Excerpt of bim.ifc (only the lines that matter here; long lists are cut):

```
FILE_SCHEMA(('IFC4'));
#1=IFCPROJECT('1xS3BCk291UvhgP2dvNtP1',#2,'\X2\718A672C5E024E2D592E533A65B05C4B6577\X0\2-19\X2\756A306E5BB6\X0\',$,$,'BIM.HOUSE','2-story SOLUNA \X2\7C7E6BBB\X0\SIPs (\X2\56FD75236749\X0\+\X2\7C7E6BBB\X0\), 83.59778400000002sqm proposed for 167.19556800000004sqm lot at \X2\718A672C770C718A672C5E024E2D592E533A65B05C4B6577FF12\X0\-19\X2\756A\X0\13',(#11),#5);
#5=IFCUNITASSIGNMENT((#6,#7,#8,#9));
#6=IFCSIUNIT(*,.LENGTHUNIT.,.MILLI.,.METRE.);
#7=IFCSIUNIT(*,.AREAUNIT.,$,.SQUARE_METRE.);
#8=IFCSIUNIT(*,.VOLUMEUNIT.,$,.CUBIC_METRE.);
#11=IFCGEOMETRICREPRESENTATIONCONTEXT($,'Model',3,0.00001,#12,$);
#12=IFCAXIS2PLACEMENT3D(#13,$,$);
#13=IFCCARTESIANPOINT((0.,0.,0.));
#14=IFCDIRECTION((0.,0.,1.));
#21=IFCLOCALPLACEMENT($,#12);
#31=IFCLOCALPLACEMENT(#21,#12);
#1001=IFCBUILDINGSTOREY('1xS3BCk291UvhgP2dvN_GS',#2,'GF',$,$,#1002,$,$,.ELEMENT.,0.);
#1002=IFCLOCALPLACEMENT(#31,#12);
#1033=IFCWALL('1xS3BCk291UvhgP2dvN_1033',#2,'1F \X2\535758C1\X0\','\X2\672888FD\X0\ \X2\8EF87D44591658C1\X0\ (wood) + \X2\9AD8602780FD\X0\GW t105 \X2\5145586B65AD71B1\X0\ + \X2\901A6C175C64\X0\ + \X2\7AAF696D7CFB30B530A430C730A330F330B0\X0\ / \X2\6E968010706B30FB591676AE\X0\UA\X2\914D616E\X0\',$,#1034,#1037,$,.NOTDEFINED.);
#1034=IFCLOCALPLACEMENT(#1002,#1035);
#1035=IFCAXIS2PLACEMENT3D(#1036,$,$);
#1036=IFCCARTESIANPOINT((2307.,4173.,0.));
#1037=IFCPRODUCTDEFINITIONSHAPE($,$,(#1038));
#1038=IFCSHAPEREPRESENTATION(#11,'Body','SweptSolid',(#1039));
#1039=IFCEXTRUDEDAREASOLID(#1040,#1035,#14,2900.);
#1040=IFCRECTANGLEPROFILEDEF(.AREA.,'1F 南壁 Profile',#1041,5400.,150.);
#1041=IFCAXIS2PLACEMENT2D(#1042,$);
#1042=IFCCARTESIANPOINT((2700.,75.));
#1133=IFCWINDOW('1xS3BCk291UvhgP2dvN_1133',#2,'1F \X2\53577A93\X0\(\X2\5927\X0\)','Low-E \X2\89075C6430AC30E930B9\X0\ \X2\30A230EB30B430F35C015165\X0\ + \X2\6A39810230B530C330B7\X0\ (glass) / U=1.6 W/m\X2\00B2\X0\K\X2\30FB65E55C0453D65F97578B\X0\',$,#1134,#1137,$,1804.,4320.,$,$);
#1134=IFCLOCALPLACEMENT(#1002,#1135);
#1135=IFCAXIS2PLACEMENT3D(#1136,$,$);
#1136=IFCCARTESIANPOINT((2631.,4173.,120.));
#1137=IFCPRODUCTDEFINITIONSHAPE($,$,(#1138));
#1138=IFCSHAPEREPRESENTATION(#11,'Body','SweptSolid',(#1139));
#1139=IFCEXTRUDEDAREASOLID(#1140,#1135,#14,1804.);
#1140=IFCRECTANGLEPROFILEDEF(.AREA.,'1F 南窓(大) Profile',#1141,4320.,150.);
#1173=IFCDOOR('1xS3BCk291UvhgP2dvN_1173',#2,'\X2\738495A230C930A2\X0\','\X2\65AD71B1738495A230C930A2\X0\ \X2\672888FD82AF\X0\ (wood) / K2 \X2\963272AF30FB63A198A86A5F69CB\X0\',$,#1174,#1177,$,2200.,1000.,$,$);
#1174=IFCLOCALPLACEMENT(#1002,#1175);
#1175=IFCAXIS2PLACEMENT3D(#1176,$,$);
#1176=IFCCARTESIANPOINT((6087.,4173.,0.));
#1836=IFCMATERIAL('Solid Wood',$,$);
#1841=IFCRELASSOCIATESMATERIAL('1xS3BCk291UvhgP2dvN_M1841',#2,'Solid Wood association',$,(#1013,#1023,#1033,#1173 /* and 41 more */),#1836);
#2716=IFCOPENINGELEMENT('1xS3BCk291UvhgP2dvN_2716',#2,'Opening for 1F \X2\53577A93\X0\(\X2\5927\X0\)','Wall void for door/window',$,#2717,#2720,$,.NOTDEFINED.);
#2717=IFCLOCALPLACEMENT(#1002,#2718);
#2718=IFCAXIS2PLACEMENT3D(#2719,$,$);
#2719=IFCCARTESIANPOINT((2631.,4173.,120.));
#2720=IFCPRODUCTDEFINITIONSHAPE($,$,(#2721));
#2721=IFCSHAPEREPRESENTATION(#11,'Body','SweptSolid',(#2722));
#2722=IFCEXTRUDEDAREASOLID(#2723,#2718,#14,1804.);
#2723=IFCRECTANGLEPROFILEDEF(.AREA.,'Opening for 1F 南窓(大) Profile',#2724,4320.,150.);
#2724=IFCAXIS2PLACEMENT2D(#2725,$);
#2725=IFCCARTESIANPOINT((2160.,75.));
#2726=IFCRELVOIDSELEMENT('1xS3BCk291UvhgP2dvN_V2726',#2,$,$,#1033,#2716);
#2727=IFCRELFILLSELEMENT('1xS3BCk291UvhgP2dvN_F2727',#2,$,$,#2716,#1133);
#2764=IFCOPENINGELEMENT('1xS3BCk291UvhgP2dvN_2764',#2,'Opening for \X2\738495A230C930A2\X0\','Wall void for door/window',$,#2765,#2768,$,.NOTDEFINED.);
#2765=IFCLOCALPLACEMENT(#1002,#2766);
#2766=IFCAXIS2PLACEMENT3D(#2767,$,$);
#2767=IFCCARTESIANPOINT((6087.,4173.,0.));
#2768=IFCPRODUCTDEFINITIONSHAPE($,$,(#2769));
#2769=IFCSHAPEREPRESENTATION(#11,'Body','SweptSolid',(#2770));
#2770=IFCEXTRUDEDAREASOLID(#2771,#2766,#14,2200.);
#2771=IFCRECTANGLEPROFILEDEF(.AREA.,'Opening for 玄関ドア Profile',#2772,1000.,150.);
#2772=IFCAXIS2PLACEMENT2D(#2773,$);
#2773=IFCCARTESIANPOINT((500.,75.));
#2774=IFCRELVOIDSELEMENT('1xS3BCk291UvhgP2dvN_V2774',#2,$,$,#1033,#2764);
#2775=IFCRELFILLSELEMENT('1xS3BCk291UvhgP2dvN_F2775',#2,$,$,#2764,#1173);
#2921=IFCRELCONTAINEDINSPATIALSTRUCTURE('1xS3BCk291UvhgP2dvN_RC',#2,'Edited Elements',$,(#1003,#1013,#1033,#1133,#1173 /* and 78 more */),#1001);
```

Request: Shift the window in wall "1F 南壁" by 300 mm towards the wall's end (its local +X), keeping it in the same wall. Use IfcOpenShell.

```python
import ifcopenshell
import ifcopenshell.api.geometry
import ifcopenshell.util.placement

model = ifcopenshell.open("bim.ifc")

window = model.by_guid("1xS3BCk291UvhgP2dvN_1133")
opening = window.FillsVoids[0].RelatingOpeningElement
wall = opening.VoidsElements[0].RelatingBuildingElement

wall_matrix = ifcopenshell.util.placement.get_local_placement(wall.ObjectPlacement)
shift = wall_matrix[:3, 0] * 300.0
before = ifcopenshell.util.placement.get_local_placement(window.ObjectPlacement)[:3, 3].copy()

# The window is not placed relative to its opening, so move both.
for product in (opening, window):
    matrix = ifcopenshell.util.placement.get_local_placement(product.ObjectPlacement)
    matrix[:3, 3] += shift
    ifcopenshell.api.geometry.edit_object_placement(model, product=product, matrix=matrix, is_si=False)

after = ifcopenshell.util.placement.get_local_placement(window.ObjectPlacement)[:3, 3]
print("window moved by", (after - before).round(3) + 0.0)

model.write("bim_v2.ifc")
```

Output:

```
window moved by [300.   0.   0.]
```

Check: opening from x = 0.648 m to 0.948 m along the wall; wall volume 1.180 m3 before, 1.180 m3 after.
